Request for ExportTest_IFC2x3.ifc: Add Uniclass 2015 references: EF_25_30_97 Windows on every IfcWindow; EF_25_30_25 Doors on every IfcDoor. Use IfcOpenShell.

First a look at what the model holds.

```python
import ifcopenshell

model = ifcopenshell.open("ExportTest_IFC2x3.ifc")
print(model.schema)
print("classifications:", [c.Name for c in model.by_type("IfcClassification")])
for ifc_class in ("IfcDoor", "IfcRoof", "IfcStair", "IfcWall", "IfcWindow"):
    print(ifc_class, len(model.by_type(ifc_class)))
```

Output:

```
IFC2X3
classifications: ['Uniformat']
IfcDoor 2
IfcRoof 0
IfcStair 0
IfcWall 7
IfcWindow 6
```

```python
import ifcopenshell
import ifcopenshell.api.classification

model = ifcopenshell.open("ExportTest_IFC2x3.ifc")

# IFC2X3 requires Source and Edition and has no link from the project to the system.
system = model.create_entity("IfcClassification", Source="NBS", Edition="2015", Name="Uniclass 2015")

codes = {
    "IfcWindow": ("EF_25_30_97", "Windows"),
    "IfcDoor": ("EF_25_30_25", "Doors"),
}
for ifc_class, (code, name) in codes.items():
    products = model.by_type(ifc_class)
    ifcopenshell.api.classification.add_reference(
        model, products=products, classification=system, identification=code, name=name
    )
    print(code, len(products))

model.write("ExportTest_IFC2x3_edited.ifc")
```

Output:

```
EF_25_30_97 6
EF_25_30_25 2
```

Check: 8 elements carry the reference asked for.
